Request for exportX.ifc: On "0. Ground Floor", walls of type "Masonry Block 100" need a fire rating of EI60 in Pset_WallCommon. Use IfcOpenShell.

First a look at what the model holds.

```python
import ifcopenshell
import ifcopenshell.util.element

model = ifcopenshell.open("exportX.ifc")
print(model.schema)
storey = next(s for s in model.by_type("IfcBuildingStorey") if s.Name == "0. Ground Floor")
walls = [e for e in ifcopenshell.util.element.get_decomposition(storey) if e.is_a("IfcWall")]
seen = {}
for e in walls:
    element_type = ifcopenshell.util.element.get_type(e)
    key = (element_type.Name if element_type != e and element_type else None, ifcopenshell.util.element.get_pset(e, "Pset_WallCommon", "FireRating"))
    seen[key] = seen.get(key, 0) + 1
for (name, value), count in sorted(seen.items(), key=str):
    print(count, "x", name, "|", value)
```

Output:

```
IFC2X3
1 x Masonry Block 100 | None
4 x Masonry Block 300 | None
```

```python
import ifcopenshell
import ifcopenshell.api.pset
import ifcopenshell.util.element

model = ifcopenshell.open("exportX.ifc")

storey = next(s for s in model.by_type("IfcBuildingStorey") if s.Name == "0. Ground Floor")
walls = [e for e in ifcopenshell.util.element.get_decomposition(storey) if e.is_a("IfcWall")]

count = 0
for e in walls:
    element_type = ifcopenshell.util.element.get_type(e)
    if element_type in (None, e) or element_type.Name != "Masonry Block 100":
        continue
    # add_pset returns the element's existing set when there is one.
    pset = ifcopenshell.api.pset.add_pset(model, product=e, name="Pset_WallCommon")
    ifcopenshell.api.pset.edit_pset(model, pset=pset, properties={"FireRating": "EI60"})
    count += 1

print(count, "walls updated")

model.write("exportX_updated.ifc")
```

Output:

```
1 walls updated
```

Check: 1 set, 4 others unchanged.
